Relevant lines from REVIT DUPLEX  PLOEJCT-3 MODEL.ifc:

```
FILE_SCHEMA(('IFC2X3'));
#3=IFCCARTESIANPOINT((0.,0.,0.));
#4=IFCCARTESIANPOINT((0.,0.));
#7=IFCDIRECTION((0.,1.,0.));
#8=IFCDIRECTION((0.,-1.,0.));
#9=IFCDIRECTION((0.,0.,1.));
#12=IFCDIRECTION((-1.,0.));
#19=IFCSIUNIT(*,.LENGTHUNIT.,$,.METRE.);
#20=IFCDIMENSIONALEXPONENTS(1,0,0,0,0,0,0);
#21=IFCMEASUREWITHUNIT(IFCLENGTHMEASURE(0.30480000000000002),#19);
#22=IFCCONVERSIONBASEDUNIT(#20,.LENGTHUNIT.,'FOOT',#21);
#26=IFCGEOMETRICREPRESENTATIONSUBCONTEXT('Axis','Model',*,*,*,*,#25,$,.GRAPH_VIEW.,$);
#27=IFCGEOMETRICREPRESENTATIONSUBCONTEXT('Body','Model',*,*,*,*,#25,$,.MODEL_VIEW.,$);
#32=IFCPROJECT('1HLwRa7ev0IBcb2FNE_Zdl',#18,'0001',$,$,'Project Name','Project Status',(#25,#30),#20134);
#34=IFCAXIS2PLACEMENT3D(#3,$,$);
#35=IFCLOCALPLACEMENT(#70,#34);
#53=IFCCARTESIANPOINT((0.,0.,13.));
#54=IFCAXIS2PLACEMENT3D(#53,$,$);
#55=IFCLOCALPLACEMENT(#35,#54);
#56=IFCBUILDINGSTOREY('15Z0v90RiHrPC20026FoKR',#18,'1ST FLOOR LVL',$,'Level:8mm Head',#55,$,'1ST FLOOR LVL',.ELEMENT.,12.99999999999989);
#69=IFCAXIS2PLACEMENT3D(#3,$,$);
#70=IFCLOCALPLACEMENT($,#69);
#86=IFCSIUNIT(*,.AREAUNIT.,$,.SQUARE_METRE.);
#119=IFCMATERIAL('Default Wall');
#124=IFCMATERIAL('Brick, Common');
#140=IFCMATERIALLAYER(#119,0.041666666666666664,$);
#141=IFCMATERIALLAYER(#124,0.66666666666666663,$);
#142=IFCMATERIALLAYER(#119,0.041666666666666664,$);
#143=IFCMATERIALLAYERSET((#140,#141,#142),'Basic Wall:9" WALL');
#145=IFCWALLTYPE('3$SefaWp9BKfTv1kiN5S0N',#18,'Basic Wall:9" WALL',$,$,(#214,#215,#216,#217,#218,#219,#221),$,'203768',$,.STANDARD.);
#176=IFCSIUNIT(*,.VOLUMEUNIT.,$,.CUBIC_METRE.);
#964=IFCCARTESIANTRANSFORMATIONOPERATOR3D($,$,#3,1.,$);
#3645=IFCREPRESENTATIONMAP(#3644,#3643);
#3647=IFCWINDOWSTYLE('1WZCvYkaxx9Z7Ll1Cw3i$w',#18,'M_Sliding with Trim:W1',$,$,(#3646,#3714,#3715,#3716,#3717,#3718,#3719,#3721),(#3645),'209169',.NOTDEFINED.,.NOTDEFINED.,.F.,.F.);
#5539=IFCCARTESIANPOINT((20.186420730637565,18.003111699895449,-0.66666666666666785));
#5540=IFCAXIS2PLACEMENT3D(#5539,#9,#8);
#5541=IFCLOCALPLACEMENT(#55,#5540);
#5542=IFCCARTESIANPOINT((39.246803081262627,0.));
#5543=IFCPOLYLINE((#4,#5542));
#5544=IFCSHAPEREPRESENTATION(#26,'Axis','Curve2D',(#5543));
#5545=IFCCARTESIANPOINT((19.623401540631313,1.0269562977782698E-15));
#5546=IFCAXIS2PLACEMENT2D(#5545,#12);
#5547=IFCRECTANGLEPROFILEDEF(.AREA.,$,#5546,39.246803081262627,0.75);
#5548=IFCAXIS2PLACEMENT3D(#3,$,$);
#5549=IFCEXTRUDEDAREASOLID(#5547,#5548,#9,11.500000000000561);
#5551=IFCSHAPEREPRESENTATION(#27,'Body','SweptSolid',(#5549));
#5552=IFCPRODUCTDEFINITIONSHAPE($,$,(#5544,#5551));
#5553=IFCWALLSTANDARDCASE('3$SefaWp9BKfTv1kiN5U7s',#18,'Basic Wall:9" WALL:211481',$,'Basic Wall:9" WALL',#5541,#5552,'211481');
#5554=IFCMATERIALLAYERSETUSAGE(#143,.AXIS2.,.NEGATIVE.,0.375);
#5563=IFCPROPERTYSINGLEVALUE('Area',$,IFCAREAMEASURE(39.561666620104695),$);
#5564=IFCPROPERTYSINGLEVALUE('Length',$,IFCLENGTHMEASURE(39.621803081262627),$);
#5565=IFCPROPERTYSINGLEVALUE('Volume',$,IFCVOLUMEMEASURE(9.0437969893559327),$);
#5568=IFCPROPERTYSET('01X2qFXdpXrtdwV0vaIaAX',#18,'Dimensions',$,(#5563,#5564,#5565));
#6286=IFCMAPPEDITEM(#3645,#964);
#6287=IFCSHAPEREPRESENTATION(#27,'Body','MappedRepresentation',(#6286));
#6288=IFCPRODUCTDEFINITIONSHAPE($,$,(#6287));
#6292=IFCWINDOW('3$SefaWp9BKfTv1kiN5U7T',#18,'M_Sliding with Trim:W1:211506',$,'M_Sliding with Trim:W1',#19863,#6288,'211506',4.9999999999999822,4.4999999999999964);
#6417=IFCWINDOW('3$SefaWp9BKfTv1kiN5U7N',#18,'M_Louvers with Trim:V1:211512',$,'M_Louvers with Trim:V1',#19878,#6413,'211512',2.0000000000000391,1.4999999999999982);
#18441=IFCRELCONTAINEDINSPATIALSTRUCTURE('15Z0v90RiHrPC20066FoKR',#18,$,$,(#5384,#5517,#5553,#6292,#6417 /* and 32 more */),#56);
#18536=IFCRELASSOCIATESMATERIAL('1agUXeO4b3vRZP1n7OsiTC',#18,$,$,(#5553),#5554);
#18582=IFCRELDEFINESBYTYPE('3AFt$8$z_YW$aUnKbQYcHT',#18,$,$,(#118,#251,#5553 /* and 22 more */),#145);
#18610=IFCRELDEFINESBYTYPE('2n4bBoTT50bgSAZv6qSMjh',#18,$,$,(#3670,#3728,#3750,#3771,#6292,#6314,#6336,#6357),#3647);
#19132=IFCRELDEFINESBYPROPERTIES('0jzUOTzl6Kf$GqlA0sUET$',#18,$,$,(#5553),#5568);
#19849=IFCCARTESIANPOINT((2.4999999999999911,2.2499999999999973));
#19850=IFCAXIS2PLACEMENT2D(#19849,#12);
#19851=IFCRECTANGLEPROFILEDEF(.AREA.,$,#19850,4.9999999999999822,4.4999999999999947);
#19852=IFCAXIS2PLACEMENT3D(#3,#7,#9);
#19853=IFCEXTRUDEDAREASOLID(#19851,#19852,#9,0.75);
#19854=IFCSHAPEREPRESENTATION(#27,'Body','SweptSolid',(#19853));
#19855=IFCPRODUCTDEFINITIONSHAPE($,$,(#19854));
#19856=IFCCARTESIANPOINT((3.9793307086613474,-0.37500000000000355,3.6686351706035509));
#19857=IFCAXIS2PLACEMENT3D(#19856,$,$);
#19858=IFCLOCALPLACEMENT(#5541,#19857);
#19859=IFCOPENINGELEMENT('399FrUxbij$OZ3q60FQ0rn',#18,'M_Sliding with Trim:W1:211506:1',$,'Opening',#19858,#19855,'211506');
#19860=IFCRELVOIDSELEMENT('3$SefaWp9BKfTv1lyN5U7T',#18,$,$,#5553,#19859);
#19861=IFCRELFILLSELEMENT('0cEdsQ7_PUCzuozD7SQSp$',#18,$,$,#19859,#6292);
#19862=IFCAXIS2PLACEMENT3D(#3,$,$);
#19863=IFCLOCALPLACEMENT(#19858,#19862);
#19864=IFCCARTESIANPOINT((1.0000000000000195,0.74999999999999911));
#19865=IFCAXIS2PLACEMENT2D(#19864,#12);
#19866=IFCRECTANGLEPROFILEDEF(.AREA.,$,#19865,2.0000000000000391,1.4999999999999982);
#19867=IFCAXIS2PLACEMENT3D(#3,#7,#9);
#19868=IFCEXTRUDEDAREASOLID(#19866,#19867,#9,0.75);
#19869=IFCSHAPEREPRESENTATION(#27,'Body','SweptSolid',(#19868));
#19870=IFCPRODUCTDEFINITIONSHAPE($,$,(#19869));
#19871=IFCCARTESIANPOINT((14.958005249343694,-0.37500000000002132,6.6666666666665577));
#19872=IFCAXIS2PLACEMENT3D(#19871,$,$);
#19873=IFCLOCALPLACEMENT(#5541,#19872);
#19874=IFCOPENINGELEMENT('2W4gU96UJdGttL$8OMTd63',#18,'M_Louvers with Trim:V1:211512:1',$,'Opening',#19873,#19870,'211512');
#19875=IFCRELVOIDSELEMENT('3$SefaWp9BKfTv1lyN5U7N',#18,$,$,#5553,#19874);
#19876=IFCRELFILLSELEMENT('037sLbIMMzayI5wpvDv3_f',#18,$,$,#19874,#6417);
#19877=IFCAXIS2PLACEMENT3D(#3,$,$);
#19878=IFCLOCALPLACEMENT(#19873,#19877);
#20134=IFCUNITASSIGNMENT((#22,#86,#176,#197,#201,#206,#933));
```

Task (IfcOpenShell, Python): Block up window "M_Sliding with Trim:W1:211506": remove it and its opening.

```python
import ifcopenshell
import ifcopenshell.api.feature
import ifcopenshell.api.pset
import ifcopenshell.api.root
import ifcopenshell.geom
import ifcopenshell.util.element
import ifcopenshell.util.shape
import ifcopenshell.util.unit

model = ifcopenshell.open("REVIT DUPLEX  PLOEJCT-3 MODEL.ifc")
area_scale = ifcopenshell.util.unit.calculate_unit_scale(model, "AREAUNIT")
volume_scale = ifcopenshell.util.unit.calculate_unit_scale(model, "VOLUMEUNIT")
settings = ifcopenshell.geom.settings()


def volume(element):
    """Net volume in cubic metres, openings subtracted."""
    shape = ifcopenshell.geom.create_shape(settings, element)
    return ifcopenshell.util.shape.get_volume(shape.geometry)


window = model.by_id(6292)
opening = window.FillsVoids[0].RelatingOpeningElement
wall = opening.VoidsElements[0].RelatingBuildingElement
before = volume(wall)

ifcopenshell.api.root.remove_product(model, product=window)
ifcopenshell.api.feature.remove_feature(model, feature=opening)

after = volume(wall)
thickness = 0.2286  # wall thickness in metres

# Update the wall's stored quantities.
pset = model.by_id(ifcopenshell.util.element.get_pset(wall, "Dimensions", should_inherit=False)["id"])
ifcopenshell.api.pset.edit_pset(model, pset=pset, properties={
    "Area": model.create_entity("IfcAreaMeasure", after / thickness / area_scale),
    "Volume": model.create_entity("IfcVolumeMeasure", after / volume_scale),
})

print(f"wall volume {before:.3f} -> {after:.3f} m3")

model.write("REVIT DUPLEX  PLOEJCT-3 MODEL_v2.ifc")
```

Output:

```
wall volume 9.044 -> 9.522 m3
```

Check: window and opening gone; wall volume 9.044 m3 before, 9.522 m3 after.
